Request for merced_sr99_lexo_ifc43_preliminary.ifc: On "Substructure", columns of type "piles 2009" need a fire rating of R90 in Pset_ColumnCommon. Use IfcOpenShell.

First a look at what the model holds.

```python
import ifcopenshell
import ifcopenshell.util.element

model = ifcopenshell.open("merced_sr99_lexo_ifc43_preliminary.ifc")
print(model.schema)
storey = next(s for s in model.by_type("IfcBuildingStorey") if s.Name == "Substructure")
columns = [e for e in ifcopenshell.util.element.get_decomposition(storey) if e.is_a("IfcColumn")]
seen = {}
for e in columns:
    element_type = ifcopenshell.util.element.get_type(e)
    key = (element_type.Name if element_type != e and element_type else None, ifcopenshell.util.element.get_pset(e, "Pset_ColumnCommon", "FireRating"))
    seen[key] = seen.get(key, 0) + 1
for (name, value), count in sorted(seen.items(), key=str):
    print(count, "x", name, "|", value)
```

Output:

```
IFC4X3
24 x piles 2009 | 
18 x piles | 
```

```python
import ifcopenshell
import ifcopenshell.api.pset
import ifcopenshell.util.element

model = ifcopenshell.open("merced_sr99_lexo_ifc43_preliminary.ifc")

storey = next(s for s in model.by_type("IfcBuildingStorey") if s.Name == "Substructure")
columns = [e for e in ifcopenshell.util.element.get_decomposition(storey) if e.is_a("IfcColumn")]

count = 0
for e in columns:
    element_type = ifcopenshell.util.element.get_type(e)
    if element_type in (None, e) or element_type.Name != "piles 2009":
        continue
    # add_pset returns the element's existing set when there is one.
    pset = ifcopenshell.api.pset.add_pset(model, product=e, name="Pset_ColumnCommon")
    ifcopenshell.api.pset.edit_pset(model, pset=pset, properties={"FireRating": "R90"})
    count += 1

print(count, "columns updated")

model.write("merced_sr99_lexo_ifc43_preliminary-out.ifc")
```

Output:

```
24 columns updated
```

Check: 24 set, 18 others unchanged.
